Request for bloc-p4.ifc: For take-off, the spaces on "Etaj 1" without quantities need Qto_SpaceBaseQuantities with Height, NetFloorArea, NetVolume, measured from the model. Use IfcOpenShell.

First a look at what the model holds.

```python
import ifcopenshell
import ifcopenshell.util.element
import ifcopenshell.util.unit

model = ifcopenshell.open("bloc-p4.ifc")
print(model.schema)
for unit_type in ("LENGTHUNIT", "AREAUNIT", "VOLUMEUNIT"):
    print(unit_type, ifcopenshell.util.unit.calculate_unit_scale(model, unit_type))
storey = next(s for s in model.by_type("IfcBuildingStorey") if s.Name == "Etaj 1")
spaces = [e for e in ifcopenshell.util.element.get_decomposition(storey) if e.is_a("IfcSpace")]
for e in sorted(spaces, key=lambda e: e.id()):
    print(e.id(), e.is_a(), e.Name, list(ifcopenshell.util.element.get_psets(e, qtos_only=True)), sep=" | ")
```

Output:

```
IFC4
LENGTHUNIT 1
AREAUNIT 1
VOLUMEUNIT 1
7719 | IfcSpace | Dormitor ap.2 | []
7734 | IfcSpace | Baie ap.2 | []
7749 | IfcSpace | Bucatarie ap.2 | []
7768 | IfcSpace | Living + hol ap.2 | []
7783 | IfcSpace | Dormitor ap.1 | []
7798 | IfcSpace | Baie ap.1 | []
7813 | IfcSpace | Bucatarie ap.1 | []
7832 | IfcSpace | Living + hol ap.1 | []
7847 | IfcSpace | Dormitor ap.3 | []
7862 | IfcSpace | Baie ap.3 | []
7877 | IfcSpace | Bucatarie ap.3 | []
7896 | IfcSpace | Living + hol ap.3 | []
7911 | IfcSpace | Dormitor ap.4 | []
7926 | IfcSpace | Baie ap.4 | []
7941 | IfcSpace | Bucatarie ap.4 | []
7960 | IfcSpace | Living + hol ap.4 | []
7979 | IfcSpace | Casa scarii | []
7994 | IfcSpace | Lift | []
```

```python
import ifcopenshell
import ifcopenshell.api.pset
import ifcopenshell.geom
import ifcopenshell.util.element
import ifcopenshell.util.shape
import ifcopenshell.util.unit

model = ifcopenshell.open("bloc-p4.ifc")
unit_scale = ifcopenshell.util.unit.calculate_unit_scale(model)
area_scale = ifcopenshell.util.unit.calculate_unit_scale(model, "AREAUNIT")
volume_scale = ifcopenshell.util.unit.calculate_unit_scale(model, "VOLUMEUNIT")
settings = ifcopenshell.geom.settings()

storey = next(s for s in model.by_type("IfcBuildingStorey") if s.Name == "Etaj 1")
spaces = [e for e in ifcopenshell.util.element.get_decomposition(storey) if e.is_a("IfcSpace")]

for e in sorted(spaces, key=lambda e: e.id()):
    if ifcopenshell.util.element.get_psets(e, qtos_only=True, should_inherit=False):
        continue
    # Geometry comes back in metres, in the element's own axes.
    shape = ifcopenshell.geom.create_shape(settings, e)
    values = {
        "Height": ifcopenshell.util.shape.get_z(shape.geometry) / unit_scale,
        "NetFloorArea": ifcopenshell.util.shape.get_footprint_area(shape.geometry) / area_scale,
        "NetVolume": ifcopenshell.util.shape.get_volume(shape.geometry) / volume_scale,
    }
    qto = ifcopenshell.api.pset.add_qto(model, product=e, name="Qto_SpaceBaseQuantities")
    ifcopenshell.api.pset.edit_qto(model, qto=qto, properties=values)
    print(e.id(), {k: round(v, 3) for k, v in values.items()})

model.write("bloc-p4_updated.ifc")
```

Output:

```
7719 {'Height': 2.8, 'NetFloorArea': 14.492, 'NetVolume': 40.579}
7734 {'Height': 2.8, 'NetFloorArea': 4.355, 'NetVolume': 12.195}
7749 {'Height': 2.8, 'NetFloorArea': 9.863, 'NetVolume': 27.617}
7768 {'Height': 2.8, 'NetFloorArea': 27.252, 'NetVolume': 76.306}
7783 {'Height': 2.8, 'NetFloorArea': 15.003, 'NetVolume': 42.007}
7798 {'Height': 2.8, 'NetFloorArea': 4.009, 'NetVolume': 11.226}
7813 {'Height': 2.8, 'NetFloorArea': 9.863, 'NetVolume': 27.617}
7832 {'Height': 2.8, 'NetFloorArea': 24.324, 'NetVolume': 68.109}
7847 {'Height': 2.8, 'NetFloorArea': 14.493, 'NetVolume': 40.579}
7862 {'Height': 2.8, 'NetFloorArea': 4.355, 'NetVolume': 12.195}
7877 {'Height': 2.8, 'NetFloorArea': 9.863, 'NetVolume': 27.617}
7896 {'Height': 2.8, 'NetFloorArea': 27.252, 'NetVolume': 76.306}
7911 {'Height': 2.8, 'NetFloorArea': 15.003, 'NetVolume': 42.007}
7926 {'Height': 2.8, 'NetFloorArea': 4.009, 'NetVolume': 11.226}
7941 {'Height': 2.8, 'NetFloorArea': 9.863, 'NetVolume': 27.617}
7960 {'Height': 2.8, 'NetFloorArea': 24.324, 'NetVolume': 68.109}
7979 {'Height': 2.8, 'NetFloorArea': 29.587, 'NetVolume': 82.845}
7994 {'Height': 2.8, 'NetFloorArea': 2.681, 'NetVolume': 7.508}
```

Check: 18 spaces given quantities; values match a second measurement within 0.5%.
